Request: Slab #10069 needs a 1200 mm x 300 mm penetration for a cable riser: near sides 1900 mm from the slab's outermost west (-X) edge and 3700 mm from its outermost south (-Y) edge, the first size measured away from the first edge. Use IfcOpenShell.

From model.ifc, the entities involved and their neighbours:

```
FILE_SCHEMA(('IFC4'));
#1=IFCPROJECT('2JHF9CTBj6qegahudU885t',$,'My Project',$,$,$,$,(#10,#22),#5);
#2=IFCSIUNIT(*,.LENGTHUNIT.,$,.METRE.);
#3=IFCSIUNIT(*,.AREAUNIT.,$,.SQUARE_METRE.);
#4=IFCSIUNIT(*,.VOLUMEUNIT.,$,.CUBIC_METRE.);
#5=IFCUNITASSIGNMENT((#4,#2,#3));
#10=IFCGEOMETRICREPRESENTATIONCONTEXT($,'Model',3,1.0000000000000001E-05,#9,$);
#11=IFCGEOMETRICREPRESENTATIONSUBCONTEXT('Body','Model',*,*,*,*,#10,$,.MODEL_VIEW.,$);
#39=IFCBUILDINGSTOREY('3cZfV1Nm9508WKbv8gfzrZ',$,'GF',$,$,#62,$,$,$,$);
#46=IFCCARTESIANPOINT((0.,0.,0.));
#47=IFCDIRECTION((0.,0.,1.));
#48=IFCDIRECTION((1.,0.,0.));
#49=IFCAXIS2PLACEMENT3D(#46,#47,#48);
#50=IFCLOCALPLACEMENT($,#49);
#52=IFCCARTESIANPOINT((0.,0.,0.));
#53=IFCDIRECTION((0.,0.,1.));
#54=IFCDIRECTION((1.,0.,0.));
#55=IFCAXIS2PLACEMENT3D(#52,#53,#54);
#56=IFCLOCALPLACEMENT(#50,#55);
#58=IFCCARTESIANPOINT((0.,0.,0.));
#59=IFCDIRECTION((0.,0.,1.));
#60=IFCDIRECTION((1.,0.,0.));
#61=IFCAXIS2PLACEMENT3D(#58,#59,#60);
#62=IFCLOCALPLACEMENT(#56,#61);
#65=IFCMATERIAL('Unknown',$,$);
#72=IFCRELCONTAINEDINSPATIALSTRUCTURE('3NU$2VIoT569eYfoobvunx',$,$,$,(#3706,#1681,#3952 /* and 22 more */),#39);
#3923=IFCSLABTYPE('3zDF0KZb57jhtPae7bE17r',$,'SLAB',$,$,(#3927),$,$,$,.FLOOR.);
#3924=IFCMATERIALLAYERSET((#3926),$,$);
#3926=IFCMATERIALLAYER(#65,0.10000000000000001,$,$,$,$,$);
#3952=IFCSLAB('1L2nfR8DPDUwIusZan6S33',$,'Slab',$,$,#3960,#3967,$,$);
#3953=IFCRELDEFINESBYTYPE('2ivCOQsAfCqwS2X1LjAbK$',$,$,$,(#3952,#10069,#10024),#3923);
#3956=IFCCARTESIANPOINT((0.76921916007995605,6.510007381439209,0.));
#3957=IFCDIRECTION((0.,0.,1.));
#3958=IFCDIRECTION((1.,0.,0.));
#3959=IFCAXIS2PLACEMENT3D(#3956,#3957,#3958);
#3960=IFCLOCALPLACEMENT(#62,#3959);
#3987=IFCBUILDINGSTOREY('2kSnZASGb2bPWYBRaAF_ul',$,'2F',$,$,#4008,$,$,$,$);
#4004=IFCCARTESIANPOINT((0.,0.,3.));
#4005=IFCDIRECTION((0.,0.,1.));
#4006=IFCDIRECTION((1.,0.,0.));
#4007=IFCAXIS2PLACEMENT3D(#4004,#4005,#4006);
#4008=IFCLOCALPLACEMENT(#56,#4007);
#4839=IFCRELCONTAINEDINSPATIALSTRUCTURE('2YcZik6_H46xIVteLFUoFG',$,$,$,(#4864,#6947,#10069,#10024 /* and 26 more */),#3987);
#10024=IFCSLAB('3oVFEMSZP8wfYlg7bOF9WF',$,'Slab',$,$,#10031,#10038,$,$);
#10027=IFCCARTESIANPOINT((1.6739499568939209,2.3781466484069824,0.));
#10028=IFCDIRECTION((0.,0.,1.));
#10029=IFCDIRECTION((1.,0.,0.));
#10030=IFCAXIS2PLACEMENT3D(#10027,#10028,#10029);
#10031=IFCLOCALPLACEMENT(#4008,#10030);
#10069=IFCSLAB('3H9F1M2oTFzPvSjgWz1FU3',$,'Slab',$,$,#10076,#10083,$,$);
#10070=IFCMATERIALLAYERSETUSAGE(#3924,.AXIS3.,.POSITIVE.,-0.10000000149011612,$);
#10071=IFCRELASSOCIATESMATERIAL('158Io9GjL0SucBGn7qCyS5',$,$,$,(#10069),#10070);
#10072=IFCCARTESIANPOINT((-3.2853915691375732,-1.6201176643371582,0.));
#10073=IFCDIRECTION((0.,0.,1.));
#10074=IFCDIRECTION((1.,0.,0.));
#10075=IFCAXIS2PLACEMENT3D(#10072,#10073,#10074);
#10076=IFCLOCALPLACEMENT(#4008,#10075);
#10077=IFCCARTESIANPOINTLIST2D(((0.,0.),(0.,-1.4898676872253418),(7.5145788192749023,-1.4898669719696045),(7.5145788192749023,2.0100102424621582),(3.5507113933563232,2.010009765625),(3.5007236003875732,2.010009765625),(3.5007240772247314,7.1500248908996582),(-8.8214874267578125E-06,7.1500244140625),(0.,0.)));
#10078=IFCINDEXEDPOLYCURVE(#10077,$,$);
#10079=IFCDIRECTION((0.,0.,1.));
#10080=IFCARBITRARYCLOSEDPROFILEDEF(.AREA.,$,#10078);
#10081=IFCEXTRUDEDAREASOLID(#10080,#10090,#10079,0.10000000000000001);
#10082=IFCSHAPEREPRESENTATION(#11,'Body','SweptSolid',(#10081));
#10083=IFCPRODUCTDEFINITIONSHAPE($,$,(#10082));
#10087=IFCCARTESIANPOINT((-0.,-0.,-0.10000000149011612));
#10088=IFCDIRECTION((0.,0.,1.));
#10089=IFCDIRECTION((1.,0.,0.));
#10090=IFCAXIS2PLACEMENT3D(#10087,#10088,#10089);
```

```python
import numpy as np
import ifcopenshell
import ifcopenshell.api.feature
import ifcopenshell.api.geometry
import ifcopenshell.api.root
import ifcopenshell.geom
import ifcopenshell.util.placement
import ifcopenshell.util.representation
import ifcopenshell.util.shape
import ifcopenshell.util.unit

model = ifcopenshell.open("model.ifc")
unit_scale = ifcopenshell.util.unit.calculate_unit_scale(model)
settings = ifcopenshell.geom.settings()


def volume(element):
    """Net volume in cubic metres, openings subtracted."""
    shape = ifcopenshell.geom.create_shape(settings, element)
    return ifcopenshell.util.shape.get_volume(shape.geometry)


slab = model.by_guid("3H9F1M2oTFzPvSjgWz1FU3")
before = volume(slab)

# Extent in the slab's own axes, in metres. The edges named are its -X and -Y sides.
slab_shape = ifcopenshell.geom.create_shape(settings, slab)
vertices = ifcopenshell.util.shape.get_vertices(slab_shape.geometry)
x_min, y_min, bottom = vertices.min(axis=0)
top = vertices[:, 2].max()

opening = ifcopenshell.api.root.create_entity(model, ifc_class="IfcOpeningElement", name="Cable riser opening", predefined_type="OPENING")
context = ifcopenshell.util.representation.get_context(model, "Model", "Body", "MODEL_VIEW")
width, depth = 1.2, 0.3
outline = [(0.0, 0.0), (width, 0.0), (width, depth), (0.0, depth), (0.0, 0.0)]
# Overshoot both faces by 50 mm so the cut is clean.
shape = ifcopenshell.api.geometry.add_slab_representation(
    model, context=context, depth=top - bottom + 0.1, polyline=outline
)
ifcopenshell.api.geometry.assign_representation(model, product=opening, representation=shape)

matrix = ifcopenshell.util.placement.get_local_placement(slab.ObjectPlacement)
matrix[:, 3] = matrix @ np.append(np.array([x_min + 1.9, y_min + 3.7, bottom - 0.05]) / unit_scale, 1.0)
ifcopenshell.api.geometry.edit_object_placement(model, product=opening, matrix=matrix, is_si=False)
ifcopenshell.api.feature.add_feature(model, feature=opening, element=slab)

after = volume(slab)

print(f"slab volume {before:.3f} -> {after:.3f} m3")

model.write("model_edited.ifc")
```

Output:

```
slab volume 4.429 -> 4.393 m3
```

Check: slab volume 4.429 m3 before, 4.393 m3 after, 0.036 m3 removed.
